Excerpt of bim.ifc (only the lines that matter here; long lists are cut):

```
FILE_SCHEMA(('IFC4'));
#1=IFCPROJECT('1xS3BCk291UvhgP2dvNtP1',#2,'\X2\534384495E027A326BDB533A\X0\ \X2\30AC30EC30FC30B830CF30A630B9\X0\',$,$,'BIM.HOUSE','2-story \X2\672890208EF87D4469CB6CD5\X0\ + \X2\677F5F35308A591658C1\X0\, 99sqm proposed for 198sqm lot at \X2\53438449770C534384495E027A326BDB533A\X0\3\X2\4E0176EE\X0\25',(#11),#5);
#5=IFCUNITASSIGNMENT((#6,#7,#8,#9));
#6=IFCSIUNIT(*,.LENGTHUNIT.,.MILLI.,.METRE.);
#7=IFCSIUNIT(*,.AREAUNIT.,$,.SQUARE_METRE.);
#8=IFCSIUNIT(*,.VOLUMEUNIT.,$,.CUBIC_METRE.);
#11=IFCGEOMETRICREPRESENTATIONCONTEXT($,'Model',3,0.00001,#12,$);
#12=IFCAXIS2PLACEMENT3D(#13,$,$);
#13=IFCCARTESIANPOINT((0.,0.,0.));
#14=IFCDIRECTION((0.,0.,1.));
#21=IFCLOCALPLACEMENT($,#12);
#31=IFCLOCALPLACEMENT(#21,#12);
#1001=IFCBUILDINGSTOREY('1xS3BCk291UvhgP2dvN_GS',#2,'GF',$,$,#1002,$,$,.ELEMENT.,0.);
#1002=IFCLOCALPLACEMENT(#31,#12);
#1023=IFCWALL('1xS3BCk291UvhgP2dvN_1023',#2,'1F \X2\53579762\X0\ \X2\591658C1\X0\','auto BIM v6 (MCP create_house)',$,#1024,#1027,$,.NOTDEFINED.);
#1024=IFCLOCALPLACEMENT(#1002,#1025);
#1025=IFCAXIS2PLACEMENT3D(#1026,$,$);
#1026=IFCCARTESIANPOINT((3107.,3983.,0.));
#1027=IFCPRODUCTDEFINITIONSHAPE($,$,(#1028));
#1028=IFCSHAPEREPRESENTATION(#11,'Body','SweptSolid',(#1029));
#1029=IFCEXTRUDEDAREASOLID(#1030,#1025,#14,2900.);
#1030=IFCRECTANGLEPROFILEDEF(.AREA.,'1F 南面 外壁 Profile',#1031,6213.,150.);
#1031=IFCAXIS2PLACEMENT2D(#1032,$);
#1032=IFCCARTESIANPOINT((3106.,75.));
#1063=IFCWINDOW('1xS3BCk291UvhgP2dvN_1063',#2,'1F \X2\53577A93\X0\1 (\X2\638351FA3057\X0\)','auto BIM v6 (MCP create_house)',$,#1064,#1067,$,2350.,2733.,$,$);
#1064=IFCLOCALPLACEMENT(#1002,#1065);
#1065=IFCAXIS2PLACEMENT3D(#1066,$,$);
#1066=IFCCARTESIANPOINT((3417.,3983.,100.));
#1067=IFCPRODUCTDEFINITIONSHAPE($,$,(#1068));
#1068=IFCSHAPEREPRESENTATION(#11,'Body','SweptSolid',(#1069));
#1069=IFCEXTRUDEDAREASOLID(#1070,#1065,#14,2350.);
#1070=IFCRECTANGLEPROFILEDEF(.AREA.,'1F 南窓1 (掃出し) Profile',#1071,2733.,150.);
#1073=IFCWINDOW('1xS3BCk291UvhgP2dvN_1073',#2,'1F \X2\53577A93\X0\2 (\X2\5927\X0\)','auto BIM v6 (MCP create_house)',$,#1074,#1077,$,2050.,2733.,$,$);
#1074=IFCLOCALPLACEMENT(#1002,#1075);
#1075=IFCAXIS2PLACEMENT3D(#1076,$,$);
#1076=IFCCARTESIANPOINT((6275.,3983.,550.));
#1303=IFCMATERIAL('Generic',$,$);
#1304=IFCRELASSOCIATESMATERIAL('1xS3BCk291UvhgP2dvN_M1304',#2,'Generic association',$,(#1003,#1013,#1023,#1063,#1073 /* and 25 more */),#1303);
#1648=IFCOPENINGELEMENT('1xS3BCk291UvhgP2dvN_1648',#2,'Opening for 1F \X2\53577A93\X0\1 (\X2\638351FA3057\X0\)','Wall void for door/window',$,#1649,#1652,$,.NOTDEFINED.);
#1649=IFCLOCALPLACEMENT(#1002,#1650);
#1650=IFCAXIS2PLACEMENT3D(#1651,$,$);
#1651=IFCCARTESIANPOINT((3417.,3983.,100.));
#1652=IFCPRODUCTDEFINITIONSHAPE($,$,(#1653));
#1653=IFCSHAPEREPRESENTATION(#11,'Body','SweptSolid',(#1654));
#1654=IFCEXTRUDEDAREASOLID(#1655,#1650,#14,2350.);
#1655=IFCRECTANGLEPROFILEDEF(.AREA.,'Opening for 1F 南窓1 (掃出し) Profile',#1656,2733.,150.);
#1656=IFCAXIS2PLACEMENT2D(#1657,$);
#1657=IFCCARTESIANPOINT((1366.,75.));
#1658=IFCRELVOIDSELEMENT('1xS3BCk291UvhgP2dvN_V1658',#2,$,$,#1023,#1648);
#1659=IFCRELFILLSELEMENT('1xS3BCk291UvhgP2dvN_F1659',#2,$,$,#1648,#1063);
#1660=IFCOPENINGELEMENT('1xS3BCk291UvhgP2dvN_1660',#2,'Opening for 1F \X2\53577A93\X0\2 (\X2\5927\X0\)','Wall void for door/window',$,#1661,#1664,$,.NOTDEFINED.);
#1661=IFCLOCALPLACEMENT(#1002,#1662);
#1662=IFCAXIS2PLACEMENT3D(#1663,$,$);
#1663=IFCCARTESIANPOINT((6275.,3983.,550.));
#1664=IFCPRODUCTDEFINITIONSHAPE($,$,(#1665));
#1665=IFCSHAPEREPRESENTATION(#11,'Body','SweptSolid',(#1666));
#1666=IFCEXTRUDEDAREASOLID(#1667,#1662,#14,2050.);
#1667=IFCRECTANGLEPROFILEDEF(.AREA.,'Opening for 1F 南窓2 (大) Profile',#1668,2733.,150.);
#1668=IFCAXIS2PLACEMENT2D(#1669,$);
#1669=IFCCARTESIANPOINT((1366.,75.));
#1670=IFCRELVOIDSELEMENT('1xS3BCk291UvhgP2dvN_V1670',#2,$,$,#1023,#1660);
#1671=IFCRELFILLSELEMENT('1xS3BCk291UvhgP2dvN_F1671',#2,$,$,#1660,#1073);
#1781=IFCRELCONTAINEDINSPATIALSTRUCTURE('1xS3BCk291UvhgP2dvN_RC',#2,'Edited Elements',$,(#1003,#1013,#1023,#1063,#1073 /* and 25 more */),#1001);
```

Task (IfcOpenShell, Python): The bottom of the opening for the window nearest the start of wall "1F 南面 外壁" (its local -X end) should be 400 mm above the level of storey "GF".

```python
import numpy as np
import ifcopenshell
import ifcopenshell.api.geometry
import ifcopenshell.geom
import ifcopenshell.util.element
import ifcopenshell.util.placement
import ifcopenshell.util.shape
import ifcopenshell.util.unit

model = ifcopenshell.open("bim.ifc")
unit_scale = ifcopenshell.util.unit.calculate_unit_scale(model)

window = model.by_id(1063)
opening = window.FillsVoids[0].RelatingOpeningElement
storey = ifcopenshell.util.element.get_container(window, ifc_class="IfcBuildingStorey")
level = ifcopenshell.util.placement.get_local_placement(storey.ObjectPlacement)[2, 3]

# The opening's origin need not be at the sill, so measure its lowest point.
shape = ifcopenshell.geom.create_shape(ifcopenshell.geom.settings(), opening)
bottom = ifcopenshell.util.shape.get_shape_bottom_elevation(shape, shape.geometry) / unit_scale
dz = level + 0.4 / unit_scale - bottom

shift = np.array([0.0, 0.0, dz])
# The window is not placed relative to its opening, so move both.
for product in (opening, window):
    matrix = ifcopenshell.util.placement.get_local_placement(product.ObjectPlacement)
    matrix[:3, 3] += shift
    ifcopenshell.api.geometry.edit_object_placement(model, product=product, matrix=matrix, is_si=False)

print(f"moved by {dz * unit_scale:+.3f} m")

model.write("bim-out.ifc")
```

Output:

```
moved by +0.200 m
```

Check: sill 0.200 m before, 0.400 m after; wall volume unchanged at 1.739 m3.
